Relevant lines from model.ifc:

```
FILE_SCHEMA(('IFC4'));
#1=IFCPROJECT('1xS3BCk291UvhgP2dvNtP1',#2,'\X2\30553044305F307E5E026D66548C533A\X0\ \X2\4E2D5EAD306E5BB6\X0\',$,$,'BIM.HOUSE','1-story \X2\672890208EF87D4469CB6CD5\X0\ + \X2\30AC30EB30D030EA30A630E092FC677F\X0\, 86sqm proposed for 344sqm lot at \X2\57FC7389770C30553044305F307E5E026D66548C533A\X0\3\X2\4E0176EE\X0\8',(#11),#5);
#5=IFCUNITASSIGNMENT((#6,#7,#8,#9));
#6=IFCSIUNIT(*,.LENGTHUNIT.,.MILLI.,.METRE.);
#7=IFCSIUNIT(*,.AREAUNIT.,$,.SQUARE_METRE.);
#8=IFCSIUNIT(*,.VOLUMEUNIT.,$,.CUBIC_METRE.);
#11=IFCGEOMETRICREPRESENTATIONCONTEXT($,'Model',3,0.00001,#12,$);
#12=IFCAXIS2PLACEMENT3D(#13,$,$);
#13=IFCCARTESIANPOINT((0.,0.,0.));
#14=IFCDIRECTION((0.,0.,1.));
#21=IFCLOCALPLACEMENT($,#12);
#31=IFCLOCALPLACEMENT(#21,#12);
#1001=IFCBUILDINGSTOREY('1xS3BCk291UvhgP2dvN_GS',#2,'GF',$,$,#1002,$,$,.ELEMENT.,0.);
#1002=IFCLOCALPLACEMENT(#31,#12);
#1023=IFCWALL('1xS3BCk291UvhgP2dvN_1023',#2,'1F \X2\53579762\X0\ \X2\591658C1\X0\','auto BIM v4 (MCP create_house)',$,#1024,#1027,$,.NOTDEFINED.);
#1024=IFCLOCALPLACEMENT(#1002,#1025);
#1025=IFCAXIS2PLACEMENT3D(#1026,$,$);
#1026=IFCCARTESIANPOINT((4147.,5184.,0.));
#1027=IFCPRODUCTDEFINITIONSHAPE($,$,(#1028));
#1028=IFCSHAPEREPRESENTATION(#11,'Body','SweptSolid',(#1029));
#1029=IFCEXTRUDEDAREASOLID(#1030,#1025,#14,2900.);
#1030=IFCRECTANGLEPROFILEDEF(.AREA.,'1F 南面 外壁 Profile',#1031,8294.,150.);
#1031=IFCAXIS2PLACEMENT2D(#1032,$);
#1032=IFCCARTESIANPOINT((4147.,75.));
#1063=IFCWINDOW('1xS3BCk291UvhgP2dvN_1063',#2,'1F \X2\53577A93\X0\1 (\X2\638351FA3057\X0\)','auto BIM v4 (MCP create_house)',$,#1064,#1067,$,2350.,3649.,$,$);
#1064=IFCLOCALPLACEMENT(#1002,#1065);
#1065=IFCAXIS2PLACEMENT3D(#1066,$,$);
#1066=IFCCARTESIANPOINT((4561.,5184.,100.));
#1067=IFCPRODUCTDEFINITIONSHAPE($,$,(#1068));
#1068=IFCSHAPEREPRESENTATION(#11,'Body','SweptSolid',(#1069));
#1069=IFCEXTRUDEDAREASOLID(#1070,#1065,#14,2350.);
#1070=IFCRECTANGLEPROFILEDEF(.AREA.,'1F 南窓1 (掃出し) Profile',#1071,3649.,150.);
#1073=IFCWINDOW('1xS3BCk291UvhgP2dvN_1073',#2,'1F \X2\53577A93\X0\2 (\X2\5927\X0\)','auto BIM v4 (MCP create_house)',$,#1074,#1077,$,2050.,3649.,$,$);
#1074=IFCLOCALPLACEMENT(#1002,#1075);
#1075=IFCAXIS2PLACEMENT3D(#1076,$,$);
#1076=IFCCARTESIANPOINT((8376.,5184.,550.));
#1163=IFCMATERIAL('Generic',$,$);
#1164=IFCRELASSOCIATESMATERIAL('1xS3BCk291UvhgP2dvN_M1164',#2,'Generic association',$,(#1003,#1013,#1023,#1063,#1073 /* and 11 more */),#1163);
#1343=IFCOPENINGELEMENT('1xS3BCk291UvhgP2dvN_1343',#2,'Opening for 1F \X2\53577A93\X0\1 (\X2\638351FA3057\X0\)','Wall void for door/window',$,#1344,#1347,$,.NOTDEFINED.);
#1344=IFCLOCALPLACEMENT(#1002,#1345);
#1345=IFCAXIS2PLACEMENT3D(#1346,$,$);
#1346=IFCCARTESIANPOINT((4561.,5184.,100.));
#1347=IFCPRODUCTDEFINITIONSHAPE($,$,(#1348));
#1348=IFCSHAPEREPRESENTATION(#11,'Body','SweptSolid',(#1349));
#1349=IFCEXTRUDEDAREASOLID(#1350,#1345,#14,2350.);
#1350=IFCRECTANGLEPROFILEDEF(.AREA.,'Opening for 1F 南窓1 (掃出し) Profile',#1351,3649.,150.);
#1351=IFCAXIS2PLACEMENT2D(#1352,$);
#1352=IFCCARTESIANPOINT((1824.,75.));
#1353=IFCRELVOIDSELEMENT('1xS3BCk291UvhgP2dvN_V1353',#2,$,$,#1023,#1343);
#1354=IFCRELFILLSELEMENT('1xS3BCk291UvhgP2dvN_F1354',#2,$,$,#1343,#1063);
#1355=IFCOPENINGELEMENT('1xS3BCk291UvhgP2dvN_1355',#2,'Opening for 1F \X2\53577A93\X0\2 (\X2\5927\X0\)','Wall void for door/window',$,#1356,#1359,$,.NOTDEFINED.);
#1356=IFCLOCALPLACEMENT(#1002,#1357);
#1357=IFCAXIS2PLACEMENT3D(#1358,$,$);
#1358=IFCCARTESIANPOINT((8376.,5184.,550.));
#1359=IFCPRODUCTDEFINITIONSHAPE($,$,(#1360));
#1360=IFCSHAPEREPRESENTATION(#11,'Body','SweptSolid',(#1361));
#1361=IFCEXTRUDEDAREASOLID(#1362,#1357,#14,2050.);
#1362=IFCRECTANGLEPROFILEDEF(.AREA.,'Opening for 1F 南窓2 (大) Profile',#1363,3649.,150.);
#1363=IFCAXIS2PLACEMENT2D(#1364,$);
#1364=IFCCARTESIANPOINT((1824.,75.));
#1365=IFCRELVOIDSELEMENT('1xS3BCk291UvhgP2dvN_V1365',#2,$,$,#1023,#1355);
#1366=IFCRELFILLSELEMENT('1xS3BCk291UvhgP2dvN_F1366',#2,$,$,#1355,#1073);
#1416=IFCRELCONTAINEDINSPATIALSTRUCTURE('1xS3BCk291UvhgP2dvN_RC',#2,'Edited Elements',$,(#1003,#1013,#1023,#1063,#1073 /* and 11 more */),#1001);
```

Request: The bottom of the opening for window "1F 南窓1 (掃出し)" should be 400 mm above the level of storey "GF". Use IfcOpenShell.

```python
import numpy as np
import ifcopenshell
import ifcopenshell.api.geometry
import ifcopenshell.geom
import ifcopenshell.util.element
import ifcopenshell.util.placement
import ifcopenshell.util.shape
import ifcopenshell.util.unit

model = ifcopenshell.open("model.ifc")
unit_scale = ifcopenshell.util.unit.calculate_unit_scale(model)

window = model.by_guid("1xS3BCk291UvhgP2dvN_1063")
opening = window.FillsVoids[0].RelatingOpeningElement
storey = ifcopenshell.util.element.get_container(window, ifc_class="IfcBuildingStorey")
level = ifcopenshell.util.placement.get_local_placement(storey.ObjectPlacement)[2, 3]

# The opening's origin need not be at the sill, so measure its lowest point.
shape = ifcopenshell.geom.create_shape(ifcopenshell.geom.settings(), opening)
bottom = ifcopenshell.util.shape.get_shape_bottom_elevation(shape, shape.geometry) / unit_scale
dz = level + 400.0 - bottom

shift = np.array([0.0, 0.0, dz])
# The window is not placed relative to its opening, so move both.
for product in (opening, window):
    matrix = ifcopenshell.util.placement.get_local_placement(product.ObjectPlacement)
    matrix[:3, 3] += shift
    ifcopenshell.api.geometry.edit_object_placement(model, product=product, matrix=matrix, is_si=False)

print(f"moved by {dz * unit_scale:+.3f} m")

model.write("model_edited.ifc")
```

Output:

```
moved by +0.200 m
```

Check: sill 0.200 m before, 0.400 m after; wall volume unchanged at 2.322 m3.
